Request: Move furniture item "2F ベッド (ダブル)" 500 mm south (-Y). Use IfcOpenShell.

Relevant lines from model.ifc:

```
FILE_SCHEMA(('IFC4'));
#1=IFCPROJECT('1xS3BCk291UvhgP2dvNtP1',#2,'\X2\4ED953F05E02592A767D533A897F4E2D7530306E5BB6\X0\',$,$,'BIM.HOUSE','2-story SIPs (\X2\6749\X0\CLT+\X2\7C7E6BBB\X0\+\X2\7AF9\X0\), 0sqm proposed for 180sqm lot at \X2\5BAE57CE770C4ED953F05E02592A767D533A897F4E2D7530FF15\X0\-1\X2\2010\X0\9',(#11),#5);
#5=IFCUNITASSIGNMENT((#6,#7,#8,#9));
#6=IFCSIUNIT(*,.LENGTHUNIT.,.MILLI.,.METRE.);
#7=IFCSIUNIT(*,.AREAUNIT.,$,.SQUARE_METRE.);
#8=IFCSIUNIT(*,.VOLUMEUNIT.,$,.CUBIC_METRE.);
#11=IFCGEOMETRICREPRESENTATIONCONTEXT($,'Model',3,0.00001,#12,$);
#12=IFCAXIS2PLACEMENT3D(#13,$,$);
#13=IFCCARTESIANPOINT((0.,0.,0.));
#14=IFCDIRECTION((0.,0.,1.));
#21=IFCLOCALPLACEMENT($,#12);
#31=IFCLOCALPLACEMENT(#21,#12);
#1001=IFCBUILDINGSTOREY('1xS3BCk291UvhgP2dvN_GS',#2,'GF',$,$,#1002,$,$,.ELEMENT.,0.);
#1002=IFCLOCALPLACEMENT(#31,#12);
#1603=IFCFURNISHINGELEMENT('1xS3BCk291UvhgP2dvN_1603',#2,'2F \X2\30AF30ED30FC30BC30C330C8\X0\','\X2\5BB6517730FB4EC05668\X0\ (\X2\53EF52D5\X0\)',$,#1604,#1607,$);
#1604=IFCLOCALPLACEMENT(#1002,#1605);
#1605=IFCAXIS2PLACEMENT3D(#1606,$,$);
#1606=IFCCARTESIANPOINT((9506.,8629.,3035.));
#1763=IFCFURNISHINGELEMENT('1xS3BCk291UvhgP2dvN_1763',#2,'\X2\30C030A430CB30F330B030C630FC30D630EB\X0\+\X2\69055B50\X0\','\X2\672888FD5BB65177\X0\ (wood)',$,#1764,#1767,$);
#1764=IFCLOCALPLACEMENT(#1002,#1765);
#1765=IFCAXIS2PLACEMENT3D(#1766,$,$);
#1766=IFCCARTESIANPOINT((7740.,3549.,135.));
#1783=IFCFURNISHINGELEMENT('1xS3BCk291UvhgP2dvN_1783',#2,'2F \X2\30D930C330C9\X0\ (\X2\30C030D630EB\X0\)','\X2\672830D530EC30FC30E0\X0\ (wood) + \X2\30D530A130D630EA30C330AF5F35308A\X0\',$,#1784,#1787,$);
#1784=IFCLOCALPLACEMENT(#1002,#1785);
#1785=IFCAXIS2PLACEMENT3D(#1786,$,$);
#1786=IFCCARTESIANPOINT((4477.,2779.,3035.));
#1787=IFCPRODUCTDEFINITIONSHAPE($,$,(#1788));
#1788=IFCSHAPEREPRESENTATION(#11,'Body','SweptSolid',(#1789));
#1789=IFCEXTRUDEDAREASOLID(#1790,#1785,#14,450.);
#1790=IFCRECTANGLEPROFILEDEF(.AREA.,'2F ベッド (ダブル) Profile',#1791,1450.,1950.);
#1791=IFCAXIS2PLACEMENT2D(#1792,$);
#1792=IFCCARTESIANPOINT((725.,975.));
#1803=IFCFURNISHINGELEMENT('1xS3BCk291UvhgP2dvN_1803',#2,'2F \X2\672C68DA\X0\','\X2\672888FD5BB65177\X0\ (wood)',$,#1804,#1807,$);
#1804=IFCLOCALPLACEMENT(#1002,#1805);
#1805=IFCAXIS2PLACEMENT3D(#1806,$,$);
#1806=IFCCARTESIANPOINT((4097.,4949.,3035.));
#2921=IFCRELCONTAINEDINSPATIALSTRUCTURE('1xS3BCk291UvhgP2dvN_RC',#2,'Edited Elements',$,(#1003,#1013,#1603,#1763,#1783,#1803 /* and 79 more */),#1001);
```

```python
import ifcopenshell
import ifcopenshell.api.geometry
import ifcopenshell.util.placement
import ifcopenshell.util.unit

model = ifcopenshell.open("model.ifc")
unit_scale = ifcopenshell.util.unit.calculate_unit_scale(model)

item = model.by_id(1783)
matrix = ifcopenshell.util.placement.get_local_placement(item.ObjectPlacement)
matrix[1, 3] -= 0.5 / unit_scale
ifcopenshell.api.geometry.edit_object_placement(model, product=item, matrix=matrix, is_si=False)

print(ifcopenshell.util.placement.get_local_placement(item.ObjectPlacement).round(3) + 0.0)

model.write("model-out.ifc")
```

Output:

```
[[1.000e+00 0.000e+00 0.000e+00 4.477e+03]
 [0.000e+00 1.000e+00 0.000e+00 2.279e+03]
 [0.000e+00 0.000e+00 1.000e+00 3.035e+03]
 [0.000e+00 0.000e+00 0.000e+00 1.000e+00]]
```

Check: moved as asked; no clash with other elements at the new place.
